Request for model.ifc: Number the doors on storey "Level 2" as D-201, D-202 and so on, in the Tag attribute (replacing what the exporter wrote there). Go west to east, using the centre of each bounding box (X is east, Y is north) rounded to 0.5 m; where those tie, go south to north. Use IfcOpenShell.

First a look at what the model holds.

```python
import ifcopenshell
import ifcopenshell.util.element
import ifcopenshell.util.placement

model = ifcopenshell.open("model.ifc")
print(model.schema)
storey = next(s for s in model.by_type("IfcBuildingStorey") if s.Name == "Level 2")
doors = [e for e in ifcopenshell.util.element.get_decomposition(storey) if e.is_a("IfcDoor")]
for e in sorted(doors, key=lambda e: e.id()):
    origin = ifcopenshell.util.placement.get_local_placement(e.ObjectPlacement)[:3, 3]
    print(e.id(), e.Tag, e.Name, origin.round(2) + 0.0, sep=" | ")
```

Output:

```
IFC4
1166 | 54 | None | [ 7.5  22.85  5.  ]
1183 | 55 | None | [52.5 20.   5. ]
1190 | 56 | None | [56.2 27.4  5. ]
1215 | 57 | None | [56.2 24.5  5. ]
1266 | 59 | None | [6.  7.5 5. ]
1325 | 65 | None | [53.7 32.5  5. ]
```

```python
import ifcopenshell
import ifcopenshell.geom
import ifcopenshell.util.element
import ifcopenshell.util.shape

model = ifcopenshell.open("model.ifc")
settings = ifcopenshell.geom.settings()
settings.set("use-world-coords", True)


def centre(element):
    shape = ifcopenshell.geom.create_shape(settings, element)
    return ifcopenshell.util.shape.get_bbox_centroid(shape.geometry)


storey = next(s for s in model.by_type("IfcBuildingStorey") if s.Name == "Level 2")
doors = [e for e in ifcopenshell.util.element.get_decomposition(storey) if e.is_a("IfcDoor")]

# Insertion points can sit at a corner or the storey origin, so sort by the geometry (in metres).
centres = {e: centre(e) for e in doors}
doors.sort(key=lambda e: (round(centres[e][0] / 0.5), centres[e][1]))

for i, e in enumerate(doors, start=1):
    number = f"D-2{i:02d}"
    e.Tag = number
    print(e.id(), number)

model.write("model_rev.ifc")
```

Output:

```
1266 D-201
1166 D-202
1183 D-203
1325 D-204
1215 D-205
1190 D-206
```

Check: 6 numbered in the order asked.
